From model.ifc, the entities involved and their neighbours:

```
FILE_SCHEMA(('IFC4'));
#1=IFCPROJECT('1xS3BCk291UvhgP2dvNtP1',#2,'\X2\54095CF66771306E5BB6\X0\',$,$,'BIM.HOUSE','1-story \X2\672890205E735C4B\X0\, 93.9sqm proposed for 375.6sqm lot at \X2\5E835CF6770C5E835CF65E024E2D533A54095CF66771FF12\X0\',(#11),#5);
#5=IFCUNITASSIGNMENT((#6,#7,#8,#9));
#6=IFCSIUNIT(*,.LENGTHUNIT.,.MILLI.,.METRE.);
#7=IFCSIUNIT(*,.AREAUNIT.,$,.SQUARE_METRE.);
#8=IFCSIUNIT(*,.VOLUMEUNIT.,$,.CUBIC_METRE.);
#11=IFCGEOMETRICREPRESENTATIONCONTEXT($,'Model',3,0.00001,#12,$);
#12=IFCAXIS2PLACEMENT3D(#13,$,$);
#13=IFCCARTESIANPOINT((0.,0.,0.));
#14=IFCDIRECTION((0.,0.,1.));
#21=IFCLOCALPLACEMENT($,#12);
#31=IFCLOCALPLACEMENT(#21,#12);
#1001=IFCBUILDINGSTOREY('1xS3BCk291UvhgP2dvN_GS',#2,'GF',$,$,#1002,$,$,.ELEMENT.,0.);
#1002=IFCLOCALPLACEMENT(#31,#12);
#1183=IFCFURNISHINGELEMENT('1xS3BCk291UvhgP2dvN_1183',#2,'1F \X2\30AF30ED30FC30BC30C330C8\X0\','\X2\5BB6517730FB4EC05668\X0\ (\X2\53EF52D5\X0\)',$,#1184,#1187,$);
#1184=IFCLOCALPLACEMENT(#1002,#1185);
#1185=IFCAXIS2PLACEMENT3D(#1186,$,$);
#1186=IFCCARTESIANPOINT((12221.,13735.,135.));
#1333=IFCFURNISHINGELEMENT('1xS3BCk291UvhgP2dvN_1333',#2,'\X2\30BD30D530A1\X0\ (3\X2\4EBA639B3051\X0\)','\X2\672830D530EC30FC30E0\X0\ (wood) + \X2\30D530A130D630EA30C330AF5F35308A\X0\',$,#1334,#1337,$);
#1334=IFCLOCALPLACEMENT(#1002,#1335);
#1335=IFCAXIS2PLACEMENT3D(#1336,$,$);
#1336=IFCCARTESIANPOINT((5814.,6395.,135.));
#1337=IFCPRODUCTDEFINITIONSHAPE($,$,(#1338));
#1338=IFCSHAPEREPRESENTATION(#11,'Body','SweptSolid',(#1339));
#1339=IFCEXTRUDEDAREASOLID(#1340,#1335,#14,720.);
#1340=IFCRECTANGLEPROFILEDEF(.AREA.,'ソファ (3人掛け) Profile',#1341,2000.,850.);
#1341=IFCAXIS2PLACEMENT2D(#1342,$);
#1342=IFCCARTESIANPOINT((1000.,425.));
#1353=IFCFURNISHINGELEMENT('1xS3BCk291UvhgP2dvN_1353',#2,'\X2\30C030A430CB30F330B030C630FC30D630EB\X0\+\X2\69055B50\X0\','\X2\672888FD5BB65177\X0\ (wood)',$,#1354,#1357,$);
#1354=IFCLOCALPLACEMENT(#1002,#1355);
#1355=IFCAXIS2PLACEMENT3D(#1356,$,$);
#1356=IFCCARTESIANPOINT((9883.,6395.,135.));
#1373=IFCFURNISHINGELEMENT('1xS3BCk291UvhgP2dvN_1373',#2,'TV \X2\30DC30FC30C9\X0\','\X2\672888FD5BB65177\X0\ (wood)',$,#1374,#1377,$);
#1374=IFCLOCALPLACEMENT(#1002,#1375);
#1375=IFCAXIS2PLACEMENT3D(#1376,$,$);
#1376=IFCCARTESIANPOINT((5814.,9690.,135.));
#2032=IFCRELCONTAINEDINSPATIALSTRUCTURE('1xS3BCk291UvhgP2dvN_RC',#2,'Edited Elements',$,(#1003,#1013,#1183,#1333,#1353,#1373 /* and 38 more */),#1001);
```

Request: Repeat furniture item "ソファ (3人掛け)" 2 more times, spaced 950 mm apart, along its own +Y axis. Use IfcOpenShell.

```python
import ifcopenshell
import ifcopenshell.api.geometry
import ifcopenshell.api.root
import ifcopenshell.util.element
import ifcopenshell.util.placement
import ifcopenshell.util.unit

model = ifcopenshell.open("model.ifc")
unit_scale = ifcopenshell.util.unit.calculate_unit_scale(model)


def reuse_history(source, copy):
    """copy_class also copies each property set's owner history, people and application; keep the originals."""
    for rel in copy.IsDefinedBy:
        if rel.is_a("IfcRelDefinesByProperties") and (history := rel.RelatingPropertyDefinition.OwnerHistory):
            rel.RelatingPropertyDefinition.OwnerHistory = source.OwnerHistory
            ifcopenshell.util.element.remove_deep2(model, history)


source = model.by_guid("1xS3BCk291UvhgP2dvN_1333")
base = ifcopenshell.util.placement.get_local_placement(source.ObjectPlacement)
step = base[:3, 1] * 0.95 / unit_scale

for i in range(1, 3):
    copy = ifcopenshell.api.root.copy_class(model, product=source)
    copy.Representation = ifcopenshell.util.element.copy_deep(
        model, source.Representation, exclude=["IfcGeometricRepresentationContext", "IfcRepresentationMap"]
    )
    reuse_history(source, copy)
    matrix = base.copy()
    matrix[:3, 3] += i * step
    print("added at", matrix[:3, 3].round(3) + 0.0)
    ifcopenshell.api.geometry.edit_object_placement(model, product=copy, matrix=matrix, is_si=False)

model.write("model_v2.ifc")
```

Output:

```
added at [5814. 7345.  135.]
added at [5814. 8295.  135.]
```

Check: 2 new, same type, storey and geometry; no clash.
